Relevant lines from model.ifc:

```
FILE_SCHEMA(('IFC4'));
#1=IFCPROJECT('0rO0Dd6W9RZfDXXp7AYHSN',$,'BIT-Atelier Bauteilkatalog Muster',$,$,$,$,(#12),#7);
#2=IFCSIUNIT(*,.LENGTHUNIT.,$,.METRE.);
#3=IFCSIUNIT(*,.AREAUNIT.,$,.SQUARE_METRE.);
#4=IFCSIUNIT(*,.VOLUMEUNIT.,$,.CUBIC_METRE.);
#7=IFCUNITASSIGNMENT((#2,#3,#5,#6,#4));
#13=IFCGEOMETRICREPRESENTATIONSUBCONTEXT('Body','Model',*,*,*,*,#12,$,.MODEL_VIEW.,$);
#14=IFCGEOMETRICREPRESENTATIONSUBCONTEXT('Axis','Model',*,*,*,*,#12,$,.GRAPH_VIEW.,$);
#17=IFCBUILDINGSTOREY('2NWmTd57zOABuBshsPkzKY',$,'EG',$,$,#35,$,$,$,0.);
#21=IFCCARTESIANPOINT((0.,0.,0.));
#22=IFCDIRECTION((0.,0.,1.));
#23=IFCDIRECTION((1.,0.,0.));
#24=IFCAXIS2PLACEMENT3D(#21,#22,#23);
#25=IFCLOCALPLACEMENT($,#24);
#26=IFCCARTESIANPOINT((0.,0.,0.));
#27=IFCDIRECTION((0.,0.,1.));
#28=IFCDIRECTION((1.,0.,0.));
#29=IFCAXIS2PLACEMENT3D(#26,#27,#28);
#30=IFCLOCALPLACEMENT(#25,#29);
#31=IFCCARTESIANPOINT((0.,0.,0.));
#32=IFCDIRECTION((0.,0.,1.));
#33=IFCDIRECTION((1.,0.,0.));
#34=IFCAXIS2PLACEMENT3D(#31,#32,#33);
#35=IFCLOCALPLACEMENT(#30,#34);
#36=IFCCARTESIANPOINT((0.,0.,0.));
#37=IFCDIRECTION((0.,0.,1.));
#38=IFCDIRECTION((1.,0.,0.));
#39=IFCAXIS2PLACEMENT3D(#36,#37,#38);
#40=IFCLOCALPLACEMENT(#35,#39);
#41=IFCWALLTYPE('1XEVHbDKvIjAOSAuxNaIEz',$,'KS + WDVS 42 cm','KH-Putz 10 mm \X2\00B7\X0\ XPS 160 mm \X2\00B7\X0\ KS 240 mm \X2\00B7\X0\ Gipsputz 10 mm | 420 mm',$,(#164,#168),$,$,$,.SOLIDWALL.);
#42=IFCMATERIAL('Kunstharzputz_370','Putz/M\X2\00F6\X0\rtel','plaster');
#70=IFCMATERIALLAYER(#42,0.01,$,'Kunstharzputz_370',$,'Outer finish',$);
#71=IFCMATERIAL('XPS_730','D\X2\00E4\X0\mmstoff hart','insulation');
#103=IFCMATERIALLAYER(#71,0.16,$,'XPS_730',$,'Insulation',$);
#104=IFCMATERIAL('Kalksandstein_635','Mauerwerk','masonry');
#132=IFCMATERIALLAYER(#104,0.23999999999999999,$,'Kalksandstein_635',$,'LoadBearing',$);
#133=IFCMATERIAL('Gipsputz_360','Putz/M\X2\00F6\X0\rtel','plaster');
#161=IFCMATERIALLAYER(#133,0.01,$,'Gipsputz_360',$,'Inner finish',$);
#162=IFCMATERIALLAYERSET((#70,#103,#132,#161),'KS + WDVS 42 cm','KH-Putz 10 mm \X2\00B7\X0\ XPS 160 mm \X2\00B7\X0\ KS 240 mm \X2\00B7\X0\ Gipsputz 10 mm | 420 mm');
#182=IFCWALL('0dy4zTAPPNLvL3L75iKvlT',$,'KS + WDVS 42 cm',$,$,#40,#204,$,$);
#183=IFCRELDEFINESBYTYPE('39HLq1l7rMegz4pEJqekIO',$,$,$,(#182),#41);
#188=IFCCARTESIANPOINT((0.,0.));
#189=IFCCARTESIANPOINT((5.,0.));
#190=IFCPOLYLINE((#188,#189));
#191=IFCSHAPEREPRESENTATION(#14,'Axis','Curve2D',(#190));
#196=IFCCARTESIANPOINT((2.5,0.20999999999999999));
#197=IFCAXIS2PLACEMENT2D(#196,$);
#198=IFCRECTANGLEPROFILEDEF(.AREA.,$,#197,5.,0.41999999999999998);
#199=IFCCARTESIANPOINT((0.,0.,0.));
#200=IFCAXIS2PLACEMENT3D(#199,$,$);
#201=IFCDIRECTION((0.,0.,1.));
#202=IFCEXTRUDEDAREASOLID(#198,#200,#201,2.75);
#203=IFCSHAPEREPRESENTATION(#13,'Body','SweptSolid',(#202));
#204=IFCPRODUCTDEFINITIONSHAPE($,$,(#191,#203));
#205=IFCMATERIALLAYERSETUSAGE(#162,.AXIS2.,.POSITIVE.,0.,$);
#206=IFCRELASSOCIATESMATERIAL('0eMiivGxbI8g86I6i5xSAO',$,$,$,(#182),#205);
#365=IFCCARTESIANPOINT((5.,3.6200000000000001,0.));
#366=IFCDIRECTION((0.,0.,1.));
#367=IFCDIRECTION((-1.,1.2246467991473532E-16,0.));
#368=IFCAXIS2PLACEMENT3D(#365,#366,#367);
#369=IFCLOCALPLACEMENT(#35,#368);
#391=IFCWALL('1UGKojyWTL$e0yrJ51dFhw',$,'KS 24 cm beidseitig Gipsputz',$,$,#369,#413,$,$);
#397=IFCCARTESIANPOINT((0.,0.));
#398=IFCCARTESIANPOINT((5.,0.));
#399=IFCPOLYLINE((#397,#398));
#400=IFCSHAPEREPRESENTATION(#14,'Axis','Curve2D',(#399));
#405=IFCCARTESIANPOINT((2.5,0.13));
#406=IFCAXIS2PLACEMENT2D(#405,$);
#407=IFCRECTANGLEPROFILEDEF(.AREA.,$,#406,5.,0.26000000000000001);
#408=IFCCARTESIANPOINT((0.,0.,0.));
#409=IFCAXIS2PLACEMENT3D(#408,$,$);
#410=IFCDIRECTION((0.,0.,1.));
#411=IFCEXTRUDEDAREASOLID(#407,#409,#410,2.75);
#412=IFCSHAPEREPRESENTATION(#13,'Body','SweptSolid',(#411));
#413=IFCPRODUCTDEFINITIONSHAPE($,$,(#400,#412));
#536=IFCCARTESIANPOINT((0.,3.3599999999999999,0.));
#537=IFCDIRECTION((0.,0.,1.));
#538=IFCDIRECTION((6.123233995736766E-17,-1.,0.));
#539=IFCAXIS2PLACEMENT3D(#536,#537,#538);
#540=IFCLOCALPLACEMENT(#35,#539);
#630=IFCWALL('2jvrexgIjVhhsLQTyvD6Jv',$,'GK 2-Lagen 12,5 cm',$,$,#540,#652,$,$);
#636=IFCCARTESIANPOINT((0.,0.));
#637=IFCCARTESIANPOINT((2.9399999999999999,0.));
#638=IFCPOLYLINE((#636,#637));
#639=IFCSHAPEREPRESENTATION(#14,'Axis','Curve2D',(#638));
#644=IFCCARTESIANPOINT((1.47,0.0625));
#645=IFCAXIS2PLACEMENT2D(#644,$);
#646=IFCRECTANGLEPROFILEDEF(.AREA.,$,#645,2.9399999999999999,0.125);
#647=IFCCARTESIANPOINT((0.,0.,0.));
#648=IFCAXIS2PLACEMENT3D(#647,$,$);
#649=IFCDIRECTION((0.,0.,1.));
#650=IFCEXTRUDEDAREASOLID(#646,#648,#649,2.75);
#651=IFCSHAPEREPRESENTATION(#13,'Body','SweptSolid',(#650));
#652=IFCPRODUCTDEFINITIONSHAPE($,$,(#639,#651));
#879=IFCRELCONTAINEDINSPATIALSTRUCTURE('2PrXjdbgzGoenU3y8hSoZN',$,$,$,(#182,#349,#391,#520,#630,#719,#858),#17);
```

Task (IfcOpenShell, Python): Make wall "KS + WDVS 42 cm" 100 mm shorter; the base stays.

```python
import ifcopenshell
import ifcopenshell.geom
import ifcopenshell.util.representation
import ifcopenshell.util.shape

model = ifcopenshell.open("model.ifc")
settings = ifcopenshell.geom.settings()


def volume(element):
    """Net volume in cubic metres, openings subtracted."""
    shape = ifcopenshell.geom.create_shape(settings, element)
    return ifcopenshell.util.shape.get_volume(shape.geometry)


wall = model.by_guid("0dy4zTAPPNLvL3L75iKvlT")
before = volume(wall)

body = ifcopenshell.util.representation.get_representation(wall, "Model", "Body")
solid = body.Items[0]
old_height = solid.Depth
solid.Depth -= 0.1
after = volume(wall)

print(f"height {old_height:g} -> {solid.Depth:g}, volume {before:.3f} -> {after:.3f} m3")

model.write("model-out.ifc")
```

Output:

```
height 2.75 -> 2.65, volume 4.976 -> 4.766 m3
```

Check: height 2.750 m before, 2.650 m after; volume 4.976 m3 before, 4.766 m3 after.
